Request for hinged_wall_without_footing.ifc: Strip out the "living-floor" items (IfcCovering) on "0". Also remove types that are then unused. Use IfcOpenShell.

First a look at what the model holds.

```python
import ifcopenshell
import ifcopenshell.util.element

model = ifcopenshell.open("hinged_wall_without_footing.ifc")
print(model.schema)
storey = next(s for s in model.by_type("IfcBuildingStorey") if s.Name == "0")
coverings = [e for e in ifcopenshell.util.element.get_decomposition(storey) if e.is_a("IfcCovering")]
seen = {}
for e in coverings:
    element_type = ifcopenshell.util.element.get_type(e)
    name = element_type.Name if element_type not in (None, e) else None
    seen[name] = seen.get(name, 0) + 1
for name, count in sorted(seen.items(), key=str):
    print(count, "x", name)
```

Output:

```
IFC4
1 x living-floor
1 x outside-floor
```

```python
import ifcopenshell
import ifcopenshell.api.root
import ifcopenshell.util.element

model = ifcopenshell.open("hinged_wall_without_footing.ifc")

storey = next(s for s in model.by_type("IfcBuildingStorey") if s.Name == "0")
coverings = [e for e in ifcopenshell.util.element.get_decomposition(storey) if e.is_a("IfcCovering")]
targets = [e for e in coverings if (t := ifcopenshell.util.element.get_type(e)) not in (None, e) and t.Name == "living-floor"]
types = {ifcopenshell.util.element.get_type(e) for e in targets} - {None, *targets}

for e in targets:
    ifcopenshell.api.root.remove_product(model, product=e)
print(len(targets), "removed")

unused = [t for t in types if not ifcopenshell.util.element.get_types(t)]
for t in unused:
    ifcopenshell.api.root.remove_product(model, product=t)
print(len(unused), "unused types removed")

model.write("hinged_wall_without_footing_edited.ifc")
```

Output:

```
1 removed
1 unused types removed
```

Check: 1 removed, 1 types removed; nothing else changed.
